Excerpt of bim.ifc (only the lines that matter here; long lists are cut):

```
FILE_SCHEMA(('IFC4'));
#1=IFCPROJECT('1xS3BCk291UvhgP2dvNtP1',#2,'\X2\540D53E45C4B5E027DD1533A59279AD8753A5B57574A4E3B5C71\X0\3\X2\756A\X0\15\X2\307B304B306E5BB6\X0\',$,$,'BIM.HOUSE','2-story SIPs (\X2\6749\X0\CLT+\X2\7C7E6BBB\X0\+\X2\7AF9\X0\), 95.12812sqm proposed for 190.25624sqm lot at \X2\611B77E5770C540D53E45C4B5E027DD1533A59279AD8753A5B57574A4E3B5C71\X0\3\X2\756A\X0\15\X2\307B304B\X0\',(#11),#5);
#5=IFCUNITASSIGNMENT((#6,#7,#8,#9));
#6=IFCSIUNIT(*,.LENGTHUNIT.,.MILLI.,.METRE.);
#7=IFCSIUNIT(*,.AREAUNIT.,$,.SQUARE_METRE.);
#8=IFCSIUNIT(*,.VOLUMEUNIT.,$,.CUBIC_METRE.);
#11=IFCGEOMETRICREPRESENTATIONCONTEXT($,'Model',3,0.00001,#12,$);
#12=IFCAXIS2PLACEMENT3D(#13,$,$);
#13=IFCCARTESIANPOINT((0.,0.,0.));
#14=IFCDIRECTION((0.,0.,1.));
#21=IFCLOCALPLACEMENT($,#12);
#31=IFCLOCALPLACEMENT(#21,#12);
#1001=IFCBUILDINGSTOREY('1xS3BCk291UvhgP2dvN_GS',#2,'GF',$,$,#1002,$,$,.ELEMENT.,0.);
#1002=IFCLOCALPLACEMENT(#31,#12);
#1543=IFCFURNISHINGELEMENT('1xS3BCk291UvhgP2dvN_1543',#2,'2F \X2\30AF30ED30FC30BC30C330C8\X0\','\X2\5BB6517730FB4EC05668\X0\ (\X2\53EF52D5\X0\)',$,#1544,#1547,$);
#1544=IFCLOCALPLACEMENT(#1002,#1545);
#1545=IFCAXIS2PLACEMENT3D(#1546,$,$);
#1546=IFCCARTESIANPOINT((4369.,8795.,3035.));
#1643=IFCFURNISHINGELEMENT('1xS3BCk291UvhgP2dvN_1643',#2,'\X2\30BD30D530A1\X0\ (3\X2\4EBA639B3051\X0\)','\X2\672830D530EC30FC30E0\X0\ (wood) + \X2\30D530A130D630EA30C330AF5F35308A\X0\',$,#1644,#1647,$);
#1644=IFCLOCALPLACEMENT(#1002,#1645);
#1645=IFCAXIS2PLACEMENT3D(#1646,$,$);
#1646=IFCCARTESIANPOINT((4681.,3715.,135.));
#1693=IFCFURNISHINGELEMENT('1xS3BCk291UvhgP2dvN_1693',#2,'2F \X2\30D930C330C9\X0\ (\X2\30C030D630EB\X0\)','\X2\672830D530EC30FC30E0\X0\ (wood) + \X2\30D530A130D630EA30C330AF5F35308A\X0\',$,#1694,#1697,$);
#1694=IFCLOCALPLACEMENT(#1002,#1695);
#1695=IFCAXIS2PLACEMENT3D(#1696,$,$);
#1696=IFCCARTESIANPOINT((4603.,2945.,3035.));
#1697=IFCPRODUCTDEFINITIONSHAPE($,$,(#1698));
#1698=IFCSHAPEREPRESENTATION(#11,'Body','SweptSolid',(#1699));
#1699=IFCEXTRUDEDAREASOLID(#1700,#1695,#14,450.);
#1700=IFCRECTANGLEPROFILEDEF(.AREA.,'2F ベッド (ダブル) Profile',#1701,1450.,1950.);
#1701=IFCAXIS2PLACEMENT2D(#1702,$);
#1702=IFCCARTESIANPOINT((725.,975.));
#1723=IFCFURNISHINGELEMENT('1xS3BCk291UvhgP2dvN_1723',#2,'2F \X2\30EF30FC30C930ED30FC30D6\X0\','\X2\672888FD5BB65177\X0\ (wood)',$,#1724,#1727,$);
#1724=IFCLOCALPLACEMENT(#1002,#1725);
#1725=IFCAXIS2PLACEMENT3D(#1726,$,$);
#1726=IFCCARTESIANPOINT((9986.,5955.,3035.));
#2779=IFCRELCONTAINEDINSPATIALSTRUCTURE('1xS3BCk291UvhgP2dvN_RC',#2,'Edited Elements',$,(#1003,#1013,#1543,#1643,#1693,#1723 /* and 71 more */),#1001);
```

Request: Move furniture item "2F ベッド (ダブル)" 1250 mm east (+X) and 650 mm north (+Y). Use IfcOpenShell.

```python
import ifcopenshell
import ifcopenshell.api.geometry
import ifcopenshell.util.placement

model = ifcopenshell.open("bim.ifc")

item = model.by_guid("1xS3BCk291UvhgP2dvN_1693")
matrix = ifcopenshell.util.placement.get_local_placement(item.ObjectPlacement)
matrix[0, 3] += 1250.0
matrix[1, 3] += 650.0
ifcopenshell.api.geometry.edit_object_placement(model, product=item, matrix=matrix, is_si=False)

print(ifcopenshell.util.placement.get_local_placement(item.ObjectPlacement).round(3) + 0.0)

model.write("bim_v2.ifc")
```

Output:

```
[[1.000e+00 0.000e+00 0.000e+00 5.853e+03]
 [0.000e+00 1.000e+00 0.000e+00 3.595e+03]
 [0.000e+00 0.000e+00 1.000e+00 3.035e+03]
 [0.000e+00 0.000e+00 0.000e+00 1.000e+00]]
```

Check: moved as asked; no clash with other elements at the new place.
